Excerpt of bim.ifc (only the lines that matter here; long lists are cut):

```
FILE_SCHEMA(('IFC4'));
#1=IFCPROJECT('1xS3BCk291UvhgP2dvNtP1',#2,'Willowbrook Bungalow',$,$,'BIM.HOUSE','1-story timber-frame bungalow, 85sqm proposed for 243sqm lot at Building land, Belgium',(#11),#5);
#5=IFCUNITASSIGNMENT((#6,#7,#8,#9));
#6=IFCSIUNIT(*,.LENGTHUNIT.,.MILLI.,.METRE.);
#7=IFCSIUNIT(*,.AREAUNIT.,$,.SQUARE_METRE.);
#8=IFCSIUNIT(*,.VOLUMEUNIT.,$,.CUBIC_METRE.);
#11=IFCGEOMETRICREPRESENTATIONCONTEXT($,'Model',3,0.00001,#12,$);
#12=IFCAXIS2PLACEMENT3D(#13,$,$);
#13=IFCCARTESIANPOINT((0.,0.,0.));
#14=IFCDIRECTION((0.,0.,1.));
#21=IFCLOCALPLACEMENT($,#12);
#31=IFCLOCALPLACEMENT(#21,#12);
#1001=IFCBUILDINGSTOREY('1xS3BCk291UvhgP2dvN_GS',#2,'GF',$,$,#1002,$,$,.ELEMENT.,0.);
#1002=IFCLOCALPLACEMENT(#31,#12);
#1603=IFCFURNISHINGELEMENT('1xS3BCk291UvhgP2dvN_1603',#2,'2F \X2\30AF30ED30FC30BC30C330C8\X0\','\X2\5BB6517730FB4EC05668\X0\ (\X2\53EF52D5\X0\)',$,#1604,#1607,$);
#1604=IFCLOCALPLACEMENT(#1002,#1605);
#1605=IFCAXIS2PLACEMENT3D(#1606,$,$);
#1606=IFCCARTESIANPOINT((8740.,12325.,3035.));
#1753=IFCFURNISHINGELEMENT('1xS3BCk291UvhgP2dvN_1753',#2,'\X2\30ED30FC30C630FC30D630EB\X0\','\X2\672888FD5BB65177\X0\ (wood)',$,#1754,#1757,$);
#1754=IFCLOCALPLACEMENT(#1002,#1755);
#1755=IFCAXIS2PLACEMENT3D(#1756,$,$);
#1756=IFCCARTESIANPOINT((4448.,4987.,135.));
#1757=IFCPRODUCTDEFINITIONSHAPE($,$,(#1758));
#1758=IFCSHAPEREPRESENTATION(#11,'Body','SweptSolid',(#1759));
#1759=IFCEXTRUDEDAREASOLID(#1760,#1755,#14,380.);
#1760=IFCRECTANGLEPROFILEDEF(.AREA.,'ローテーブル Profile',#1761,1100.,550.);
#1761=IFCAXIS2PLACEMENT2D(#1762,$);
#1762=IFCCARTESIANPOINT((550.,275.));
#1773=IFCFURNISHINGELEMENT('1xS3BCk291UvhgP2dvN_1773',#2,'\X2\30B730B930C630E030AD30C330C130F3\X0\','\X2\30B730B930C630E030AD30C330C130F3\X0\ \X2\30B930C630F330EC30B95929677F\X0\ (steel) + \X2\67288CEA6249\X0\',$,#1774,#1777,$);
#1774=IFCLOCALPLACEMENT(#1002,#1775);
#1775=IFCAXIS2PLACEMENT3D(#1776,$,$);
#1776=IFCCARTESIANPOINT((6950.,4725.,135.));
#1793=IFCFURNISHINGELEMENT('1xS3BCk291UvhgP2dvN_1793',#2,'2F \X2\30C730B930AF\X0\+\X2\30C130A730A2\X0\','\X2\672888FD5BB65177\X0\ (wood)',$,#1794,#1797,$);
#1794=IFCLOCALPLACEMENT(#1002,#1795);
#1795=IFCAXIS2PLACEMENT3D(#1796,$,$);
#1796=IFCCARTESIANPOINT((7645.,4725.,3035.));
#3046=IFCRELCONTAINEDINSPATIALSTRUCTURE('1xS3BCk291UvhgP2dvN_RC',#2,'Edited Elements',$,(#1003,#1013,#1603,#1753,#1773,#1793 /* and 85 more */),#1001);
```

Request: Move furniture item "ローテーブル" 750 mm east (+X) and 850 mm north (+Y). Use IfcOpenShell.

```python
import ifcopenshell
import ifcopenshell.api.geometry
import ifcopenshell.util.placement
import ifcopenshell.util.unit

model = ifcopenshell.open("bim.ifc")
unit_scale = ifcopenshell.util.unit.calculate_unit_scale(model)

item = model.by_guid("1xS3BCk291UvhgP2dvN_1753")
matrix = ifcopenshell.util.placement.get_local_placement(item.ObjectPlacement)
matrix[0, 3] += 0.75 / unit_scale
matrix[1, 3] += 0.85 / unit_scale
ifcopenshell.api.geometry.edit_object_placement(model, product=item, matrix=matrix, is_si=False)

print(ifcopenshell.util.placement.get_local_placement(item.ObjectPlacement).round(3) + 0.0)

model.write("bim_updated.ifc")
```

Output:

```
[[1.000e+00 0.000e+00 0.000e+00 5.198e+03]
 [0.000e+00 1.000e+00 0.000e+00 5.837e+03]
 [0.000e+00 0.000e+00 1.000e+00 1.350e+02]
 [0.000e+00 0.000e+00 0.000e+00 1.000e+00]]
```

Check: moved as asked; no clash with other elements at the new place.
